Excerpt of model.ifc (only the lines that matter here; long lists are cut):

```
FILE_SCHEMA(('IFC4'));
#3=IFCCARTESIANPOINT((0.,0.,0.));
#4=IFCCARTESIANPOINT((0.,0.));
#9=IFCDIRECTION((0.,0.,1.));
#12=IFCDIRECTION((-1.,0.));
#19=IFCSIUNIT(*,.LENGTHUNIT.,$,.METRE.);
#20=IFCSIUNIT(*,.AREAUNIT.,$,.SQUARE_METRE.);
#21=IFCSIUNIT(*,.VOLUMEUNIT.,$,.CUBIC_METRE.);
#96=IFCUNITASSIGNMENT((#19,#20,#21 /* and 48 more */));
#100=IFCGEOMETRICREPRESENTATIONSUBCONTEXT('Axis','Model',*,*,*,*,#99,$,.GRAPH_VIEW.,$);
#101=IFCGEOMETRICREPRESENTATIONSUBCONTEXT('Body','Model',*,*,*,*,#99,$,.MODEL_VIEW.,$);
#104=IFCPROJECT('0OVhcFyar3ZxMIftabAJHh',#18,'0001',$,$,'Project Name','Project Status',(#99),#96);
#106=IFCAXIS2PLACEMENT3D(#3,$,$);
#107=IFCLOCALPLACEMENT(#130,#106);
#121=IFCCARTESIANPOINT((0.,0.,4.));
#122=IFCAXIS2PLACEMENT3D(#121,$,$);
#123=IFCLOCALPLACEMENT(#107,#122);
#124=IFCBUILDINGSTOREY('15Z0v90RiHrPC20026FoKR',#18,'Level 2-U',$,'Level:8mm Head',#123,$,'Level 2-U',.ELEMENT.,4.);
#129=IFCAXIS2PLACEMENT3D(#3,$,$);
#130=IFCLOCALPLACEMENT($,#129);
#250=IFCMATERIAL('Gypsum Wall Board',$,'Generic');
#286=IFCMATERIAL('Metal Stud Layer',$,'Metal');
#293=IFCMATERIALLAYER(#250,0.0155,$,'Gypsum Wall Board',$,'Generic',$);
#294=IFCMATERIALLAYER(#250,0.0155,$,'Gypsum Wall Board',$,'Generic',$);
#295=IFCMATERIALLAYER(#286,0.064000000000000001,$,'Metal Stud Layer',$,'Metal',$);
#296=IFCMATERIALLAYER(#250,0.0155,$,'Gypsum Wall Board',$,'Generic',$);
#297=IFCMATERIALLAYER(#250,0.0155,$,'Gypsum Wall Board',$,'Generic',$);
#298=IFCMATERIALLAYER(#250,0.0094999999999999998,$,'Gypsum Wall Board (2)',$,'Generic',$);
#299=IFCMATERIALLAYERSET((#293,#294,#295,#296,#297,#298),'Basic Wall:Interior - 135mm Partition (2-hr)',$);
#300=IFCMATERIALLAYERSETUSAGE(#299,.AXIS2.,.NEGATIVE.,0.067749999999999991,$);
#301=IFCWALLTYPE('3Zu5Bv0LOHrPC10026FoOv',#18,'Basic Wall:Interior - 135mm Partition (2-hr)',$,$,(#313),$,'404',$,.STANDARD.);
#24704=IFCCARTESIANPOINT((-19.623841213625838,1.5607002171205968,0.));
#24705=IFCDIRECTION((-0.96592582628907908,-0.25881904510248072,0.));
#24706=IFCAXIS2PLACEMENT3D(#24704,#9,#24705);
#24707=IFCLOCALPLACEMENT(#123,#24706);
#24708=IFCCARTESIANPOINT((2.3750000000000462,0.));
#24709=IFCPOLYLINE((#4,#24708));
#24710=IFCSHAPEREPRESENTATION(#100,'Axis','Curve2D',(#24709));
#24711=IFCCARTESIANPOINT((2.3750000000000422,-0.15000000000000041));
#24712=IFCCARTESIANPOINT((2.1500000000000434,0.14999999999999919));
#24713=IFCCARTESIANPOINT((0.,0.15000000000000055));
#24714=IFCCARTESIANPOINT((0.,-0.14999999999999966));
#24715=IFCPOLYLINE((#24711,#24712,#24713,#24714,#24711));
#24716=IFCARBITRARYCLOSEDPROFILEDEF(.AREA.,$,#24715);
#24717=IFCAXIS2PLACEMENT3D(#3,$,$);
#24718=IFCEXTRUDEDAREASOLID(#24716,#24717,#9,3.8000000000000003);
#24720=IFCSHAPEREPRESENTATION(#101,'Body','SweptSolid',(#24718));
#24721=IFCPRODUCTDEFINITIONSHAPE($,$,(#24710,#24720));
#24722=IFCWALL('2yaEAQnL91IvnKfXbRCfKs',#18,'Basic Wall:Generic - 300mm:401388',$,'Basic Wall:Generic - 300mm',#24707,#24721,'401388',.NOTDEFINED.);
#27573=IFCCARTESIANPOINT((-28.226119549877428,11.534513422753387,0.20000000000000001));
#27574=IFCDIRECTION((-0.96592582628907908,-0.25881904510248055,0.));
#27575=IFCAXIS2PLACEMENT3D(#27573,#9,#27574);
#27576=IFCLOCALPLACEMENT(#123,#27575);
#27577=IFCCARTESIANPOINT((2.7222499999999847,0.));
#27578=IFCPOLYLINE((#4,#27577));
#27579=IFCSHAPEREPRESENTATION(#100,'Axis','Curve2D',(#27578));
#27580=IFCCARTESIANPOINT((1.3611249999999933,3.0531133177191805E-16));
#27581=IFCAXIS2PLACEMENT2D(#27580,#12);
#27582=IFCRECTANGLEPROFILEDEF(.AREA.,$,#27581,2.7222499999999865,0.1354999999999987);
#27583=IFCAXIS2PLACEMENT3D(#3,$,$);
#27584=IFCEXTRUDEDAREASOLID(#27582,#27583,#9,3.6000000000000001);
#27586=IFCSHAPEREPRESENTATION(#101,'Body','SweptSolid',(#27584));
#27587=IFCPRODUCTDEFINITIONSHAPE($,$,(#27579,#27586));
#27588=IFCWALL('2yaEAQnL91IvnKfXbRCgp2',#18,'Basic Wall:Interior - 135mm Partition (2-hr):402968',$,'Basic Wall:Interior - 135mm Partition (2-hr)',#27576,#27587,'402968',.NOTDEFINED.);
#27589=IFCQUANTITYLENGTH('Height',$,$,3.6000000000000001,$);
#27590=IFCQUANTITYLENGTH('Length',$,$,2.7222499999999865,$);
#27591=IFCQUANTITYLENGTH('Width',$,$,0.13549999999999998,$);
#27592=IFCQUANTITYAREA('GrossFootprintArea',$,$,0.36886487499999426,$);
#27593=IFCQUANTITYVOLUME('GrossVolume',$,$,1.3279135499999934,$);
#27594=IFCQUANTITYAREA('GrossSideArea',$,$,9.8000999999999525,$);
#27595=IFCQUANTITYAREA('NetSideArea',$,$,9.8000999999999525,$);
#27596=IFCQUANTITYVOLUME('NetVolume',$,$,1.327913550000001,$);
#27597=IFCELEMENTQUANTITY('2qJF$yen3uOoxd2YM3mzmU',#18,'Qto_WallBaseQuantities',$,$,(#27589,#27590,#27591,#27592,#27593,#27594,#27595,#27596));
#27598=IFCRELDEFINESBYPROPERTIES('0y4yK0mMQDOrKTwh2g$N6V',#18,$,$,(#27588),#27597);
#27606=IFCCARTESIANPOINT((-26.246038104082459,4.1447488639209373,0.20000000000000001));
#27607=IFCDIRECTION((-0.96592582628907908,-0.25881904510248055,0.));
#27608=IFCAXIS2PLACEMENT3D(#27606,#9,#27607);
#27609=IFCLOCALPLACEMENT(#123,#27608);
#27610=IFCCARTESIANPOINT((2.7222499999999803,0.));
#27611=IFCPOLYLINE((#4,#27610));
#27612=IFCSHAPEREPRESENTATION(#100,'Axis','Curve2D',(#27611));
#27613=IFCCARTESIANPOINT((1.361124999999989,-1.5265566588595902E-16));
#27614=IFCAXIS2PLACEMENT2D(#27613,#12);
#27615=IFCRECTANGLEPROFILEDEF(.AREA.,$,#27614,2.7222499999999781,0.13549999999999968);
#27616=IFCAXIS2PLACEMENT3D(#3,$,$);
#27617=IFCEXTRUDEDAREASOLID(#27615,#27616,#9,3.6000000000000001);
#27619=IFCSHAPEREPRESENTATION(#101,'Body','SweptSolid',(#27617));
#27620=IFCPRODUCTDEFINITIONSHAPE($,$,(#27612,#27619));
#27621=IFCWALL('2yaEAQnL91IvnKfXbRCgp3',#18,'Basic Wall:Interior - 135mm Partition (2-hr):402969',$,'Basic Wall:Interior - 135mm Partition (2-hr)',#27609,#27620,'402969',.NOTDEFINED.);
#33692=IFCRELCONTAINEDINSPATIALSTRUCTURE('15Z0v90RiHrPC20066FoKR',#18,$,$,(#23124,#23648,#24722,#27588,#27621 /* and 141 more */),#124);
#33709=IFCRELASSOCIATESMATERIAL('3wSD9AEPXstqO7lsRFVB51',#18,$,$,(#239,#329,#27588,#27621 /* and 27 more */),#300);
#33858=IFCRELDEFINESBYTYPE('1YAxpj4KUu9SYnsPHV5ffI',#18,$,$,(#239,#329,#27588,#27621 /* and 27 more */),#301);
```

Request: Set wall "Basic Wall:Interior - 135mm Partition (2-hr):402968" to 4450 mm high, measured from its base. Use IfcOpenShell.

```python
import ifcopenshell
import ifcopenshell.api.pset
import ifcopenshell.geom
import ifcopenshell.util.element
import ifcopenshell.util.representation
import ifcopenshell.util.shape
import ifcopenshell.util.unit

model = ifcopenshell.open("model.ifc")
unit_scale = ifcopenshell.util.unit.calculate_unit_scale(model)
area_scale = ifcopenshell.util.unit.calculate_unit_scale(model, "AREAUNIT")
volume_scale = ifcopenshell.util.unit.calculate_unit_scale(model, "VOLUMEUNIT")
settings = ifcopenshell.geom.settings()


def volume(element):
    """Net volume in cubic metres, openings subtracted."""
    shape = ifcopenshell.geom.create_shape(settings, element)
    return ifcopenshell.util.shape.get_volume(shape.geometry)


wall = model.by_id(27588)
before = volume(wall)

body = ifcopenshell.util.representation.get_representation(wall, "Model", "Body")
solid = body.Items[0]
old_height = solid.Depth
solid.Depth = 4.45
after = volume(wall)
thickness = 0.1355  # wall thickness in metres

# Update the stored height, areas and volumes.
qto = model.by_id(ifcopenshell.util.element.get_pset(wall, "Qto_WallBaseQuantities", should_inherit=False)["id"])
ifcopenshell.api.pset.edit_qto(model, qto=qto, properties={
    "Height": solid.Depth,
    "GrossVolume": ifcopenshell.util.element.get_pset(wall, "Qto_WallBaseQuantities", "GrossVolume") * solid.Depth / old_height,
    "GrossSideArea": ifcopenshell.util.element.get_pset(wall, "Qto_WallBaseQuantities", "GrossSideArea") * solid.Depth / old_height,
    "NetSideArea": after / thickness / area_scale,
    "NetVolume": after / volume_scale,
})

print(f"height {old_height:g} -> {solid.Depth:g}, volume {before:.3f} -> {after:.3f} m3")

model.write("model_edited.ifc")
```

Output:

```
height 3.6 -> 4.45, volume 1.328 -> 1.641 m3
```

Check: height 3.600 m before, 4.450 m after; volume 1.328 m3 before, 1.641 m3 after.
